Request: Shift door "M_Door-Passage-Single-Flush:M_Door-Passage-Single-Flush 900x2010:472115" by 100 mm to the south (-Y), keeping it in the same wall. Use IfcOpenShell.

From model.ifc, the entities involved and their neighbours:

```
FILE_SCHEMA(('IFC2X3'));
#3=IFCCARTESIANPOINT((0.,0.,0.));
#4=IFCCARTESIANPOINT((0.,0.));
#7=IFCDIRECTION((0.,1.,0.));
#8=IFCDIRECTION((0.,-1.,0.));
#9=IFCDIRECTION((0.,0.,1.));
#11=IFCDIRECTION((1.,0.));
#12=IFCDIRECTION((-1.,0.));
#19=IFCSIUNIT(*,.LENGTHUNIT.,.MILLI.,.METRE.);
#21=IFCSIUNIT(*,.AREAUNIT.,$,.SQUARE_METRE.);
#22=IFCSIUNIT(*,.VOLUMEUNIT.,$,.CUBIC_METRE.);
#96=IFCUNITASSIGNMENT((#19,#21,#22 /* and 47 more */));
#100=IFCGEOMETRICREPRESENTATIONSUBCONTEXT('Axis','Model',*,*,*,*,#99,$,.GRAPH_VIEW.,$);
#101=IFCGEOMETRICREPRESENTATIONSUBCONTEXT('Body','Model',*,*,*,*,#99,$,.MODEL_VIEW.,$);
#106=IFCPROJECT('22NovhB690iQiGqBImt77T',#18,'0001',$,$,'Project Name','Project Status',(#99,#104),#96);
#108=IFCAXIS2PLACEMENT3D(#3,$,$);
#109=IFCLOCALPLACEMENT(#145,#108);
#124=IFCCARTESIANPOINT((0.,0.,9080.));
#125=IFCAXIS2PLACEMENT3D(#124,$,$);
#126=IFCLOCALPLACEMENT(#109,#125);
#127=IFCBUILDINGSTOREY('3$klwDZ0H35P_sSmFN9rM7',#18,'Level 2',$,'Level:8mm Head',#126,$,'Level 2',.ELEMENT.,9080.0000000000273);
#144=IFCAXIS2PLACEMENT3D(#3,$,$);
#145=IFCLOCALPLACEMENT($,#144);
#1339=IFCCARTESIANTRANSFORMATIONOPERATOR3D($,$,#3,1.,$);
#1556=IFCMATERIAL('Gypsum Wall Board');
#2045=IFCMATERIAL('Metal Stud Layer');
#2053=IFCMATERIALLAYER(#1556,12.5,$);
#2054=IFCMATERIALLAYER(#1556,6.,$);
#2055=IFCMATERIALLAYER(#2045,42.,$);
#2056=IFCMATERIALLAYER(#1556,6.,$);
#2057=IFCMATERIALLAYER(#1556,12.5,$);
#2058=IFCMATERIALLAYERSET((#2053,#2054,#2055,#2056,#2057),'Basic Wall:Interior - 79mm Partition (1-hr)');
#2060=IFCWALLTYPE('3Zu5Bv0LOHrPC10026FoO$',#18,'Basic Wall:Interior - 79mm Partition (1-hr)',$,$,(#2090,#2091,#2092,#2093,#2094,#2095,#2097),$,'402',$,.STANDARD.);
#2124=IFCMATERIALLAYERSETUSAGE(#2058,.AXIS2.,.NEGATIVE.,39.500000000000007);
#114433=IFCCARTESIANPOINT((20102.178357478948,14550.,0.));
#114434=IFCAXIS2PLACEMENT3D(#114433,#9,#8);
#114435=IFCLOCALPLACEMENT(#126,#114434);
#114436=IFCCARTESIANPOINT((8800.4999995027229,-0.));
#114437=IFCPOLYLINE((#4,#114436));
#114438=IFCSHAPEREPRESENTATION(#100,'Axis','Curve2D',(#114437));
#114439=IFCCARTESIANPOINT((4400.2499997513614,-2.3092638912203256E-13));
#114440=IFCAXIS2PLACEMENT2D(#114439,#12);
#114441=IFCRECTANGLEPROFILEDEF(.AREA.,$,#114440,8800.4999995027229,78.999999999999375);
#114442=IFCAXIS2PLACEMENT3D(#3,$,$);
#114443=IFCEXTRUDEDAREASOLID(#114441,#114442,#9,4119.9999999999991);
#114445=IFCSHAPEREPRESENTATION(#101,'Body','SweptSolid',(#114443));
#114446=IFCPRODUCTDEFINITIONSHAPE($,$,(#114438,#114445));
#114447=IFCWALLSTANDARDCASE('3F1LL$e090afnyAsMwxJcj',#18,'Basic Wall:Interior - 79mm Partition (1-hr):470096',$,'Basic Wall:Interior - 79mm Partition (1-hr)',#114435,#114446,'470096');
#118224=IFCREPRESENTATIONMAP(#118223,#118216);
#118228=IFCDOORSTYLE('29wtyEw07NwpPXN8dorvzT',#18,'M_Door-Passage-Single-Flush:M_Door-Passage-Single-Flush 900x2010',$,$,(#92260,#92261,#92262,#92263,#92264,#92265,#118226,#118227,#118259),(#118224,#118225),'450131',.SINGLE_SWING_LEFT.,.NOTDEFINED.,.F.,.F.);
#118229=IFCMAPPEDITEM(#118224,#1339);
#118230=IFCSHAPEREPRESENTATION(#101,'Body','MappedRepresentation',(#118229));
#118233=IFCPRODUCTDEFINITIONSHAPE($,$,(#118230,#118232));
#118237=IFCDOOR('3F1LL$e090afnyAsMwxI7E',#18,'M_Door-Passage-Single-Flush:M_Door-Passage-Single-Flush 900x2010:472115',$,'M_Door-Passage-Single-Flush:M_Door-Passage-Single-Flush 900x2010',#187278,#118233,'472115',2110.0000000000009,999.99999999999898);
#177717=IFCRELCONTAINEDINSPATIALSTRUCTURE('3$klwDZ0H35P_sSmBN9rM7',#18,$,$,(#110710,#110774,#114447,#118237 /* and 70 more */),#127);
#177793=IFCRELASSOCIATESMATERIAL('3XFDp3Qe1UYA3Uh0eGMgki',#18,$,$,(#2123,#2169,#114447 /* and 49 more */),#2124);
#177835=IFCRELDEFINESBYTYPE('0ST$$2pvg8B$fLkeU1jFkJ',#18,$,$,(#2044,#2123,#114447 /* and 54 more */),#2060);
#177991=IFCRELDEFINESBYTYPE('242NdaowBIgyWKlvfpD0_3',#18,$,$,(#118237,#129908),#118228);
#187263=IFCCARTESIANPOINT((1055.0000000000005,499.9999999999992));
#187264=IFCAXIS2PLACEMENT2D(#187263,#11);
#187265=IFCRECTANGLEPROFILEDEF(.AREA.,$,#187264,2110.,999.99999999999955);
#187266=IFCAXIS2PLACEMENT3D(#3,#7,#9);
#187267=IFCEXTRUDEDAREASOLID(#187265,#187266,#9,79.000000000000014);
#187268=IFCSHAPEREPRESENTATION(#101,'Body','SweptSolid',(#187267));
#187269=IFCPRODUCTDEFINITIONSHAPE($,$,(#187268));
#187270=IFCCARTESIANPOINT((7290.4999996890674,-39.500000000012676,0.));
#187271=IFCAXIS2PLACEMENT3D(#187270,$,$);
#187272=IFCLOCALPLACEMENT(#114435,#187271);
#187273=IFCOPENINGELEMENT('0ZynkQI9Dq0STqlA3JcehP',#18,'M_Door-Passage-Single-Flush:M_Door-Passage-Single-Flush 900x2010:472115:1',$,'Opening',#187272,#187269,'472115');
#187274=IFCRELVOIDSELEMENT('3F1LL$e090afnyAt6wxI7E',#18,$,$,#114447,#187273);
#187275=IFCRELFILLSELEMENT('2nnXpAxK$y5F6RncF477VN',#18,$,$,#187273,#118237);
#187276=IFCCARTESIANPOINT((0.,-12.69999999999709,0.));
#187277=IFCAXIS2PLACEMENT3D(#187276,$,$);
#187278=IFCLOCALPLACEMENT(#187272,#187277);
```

```python
import ifcopenshell
import ifcopenshell.api.geometry
import ifcopenshell.util.placement
import ifcopenshell.util.unit

model = ifcopenshell.open("model.ifc")
unit_scale = ifcopenshell.util.unit.calculate_unit_scale(model)

door = model.by_id(118237)
opening = door.FillsVoids[0].RelatingOpeningElement
wall = opening.VoidsElements[0].RelatingBuildingElement

wall_matrix = ifcopenshell.util.placement.get_local_placement(wall.ObjectPlacement)
shift = wall_matrix[:3, 0] * 0.1 / unit_scale
before = ifcopenshell.util.placement.get_local_placement(door.ObjectPlacement)[:3, 3].copy()

# The door is placed relative to its opening, so it follows when the opening moves.
matrix = ifcopenshell.util.placement.get_local_placement(opening.ObjectPlacement)
matrix[:3, 3] += shift
ifcopenshell.api.geometry.edit_object_placement(
    model, product=opening, matrix=matrix, is_si=False, should_transform_children=True
)

after = ifcopenshell.util.placement.get_local_placement(door.ObjectPlacement)[:3, 3]
print("door moved by", (after - before).round(3) + 0.0)

model.write("model_edited.ifc")
```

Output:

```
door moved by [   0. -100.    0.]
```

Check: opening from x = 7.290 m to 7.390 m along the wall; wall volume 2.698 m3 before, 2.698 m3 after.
